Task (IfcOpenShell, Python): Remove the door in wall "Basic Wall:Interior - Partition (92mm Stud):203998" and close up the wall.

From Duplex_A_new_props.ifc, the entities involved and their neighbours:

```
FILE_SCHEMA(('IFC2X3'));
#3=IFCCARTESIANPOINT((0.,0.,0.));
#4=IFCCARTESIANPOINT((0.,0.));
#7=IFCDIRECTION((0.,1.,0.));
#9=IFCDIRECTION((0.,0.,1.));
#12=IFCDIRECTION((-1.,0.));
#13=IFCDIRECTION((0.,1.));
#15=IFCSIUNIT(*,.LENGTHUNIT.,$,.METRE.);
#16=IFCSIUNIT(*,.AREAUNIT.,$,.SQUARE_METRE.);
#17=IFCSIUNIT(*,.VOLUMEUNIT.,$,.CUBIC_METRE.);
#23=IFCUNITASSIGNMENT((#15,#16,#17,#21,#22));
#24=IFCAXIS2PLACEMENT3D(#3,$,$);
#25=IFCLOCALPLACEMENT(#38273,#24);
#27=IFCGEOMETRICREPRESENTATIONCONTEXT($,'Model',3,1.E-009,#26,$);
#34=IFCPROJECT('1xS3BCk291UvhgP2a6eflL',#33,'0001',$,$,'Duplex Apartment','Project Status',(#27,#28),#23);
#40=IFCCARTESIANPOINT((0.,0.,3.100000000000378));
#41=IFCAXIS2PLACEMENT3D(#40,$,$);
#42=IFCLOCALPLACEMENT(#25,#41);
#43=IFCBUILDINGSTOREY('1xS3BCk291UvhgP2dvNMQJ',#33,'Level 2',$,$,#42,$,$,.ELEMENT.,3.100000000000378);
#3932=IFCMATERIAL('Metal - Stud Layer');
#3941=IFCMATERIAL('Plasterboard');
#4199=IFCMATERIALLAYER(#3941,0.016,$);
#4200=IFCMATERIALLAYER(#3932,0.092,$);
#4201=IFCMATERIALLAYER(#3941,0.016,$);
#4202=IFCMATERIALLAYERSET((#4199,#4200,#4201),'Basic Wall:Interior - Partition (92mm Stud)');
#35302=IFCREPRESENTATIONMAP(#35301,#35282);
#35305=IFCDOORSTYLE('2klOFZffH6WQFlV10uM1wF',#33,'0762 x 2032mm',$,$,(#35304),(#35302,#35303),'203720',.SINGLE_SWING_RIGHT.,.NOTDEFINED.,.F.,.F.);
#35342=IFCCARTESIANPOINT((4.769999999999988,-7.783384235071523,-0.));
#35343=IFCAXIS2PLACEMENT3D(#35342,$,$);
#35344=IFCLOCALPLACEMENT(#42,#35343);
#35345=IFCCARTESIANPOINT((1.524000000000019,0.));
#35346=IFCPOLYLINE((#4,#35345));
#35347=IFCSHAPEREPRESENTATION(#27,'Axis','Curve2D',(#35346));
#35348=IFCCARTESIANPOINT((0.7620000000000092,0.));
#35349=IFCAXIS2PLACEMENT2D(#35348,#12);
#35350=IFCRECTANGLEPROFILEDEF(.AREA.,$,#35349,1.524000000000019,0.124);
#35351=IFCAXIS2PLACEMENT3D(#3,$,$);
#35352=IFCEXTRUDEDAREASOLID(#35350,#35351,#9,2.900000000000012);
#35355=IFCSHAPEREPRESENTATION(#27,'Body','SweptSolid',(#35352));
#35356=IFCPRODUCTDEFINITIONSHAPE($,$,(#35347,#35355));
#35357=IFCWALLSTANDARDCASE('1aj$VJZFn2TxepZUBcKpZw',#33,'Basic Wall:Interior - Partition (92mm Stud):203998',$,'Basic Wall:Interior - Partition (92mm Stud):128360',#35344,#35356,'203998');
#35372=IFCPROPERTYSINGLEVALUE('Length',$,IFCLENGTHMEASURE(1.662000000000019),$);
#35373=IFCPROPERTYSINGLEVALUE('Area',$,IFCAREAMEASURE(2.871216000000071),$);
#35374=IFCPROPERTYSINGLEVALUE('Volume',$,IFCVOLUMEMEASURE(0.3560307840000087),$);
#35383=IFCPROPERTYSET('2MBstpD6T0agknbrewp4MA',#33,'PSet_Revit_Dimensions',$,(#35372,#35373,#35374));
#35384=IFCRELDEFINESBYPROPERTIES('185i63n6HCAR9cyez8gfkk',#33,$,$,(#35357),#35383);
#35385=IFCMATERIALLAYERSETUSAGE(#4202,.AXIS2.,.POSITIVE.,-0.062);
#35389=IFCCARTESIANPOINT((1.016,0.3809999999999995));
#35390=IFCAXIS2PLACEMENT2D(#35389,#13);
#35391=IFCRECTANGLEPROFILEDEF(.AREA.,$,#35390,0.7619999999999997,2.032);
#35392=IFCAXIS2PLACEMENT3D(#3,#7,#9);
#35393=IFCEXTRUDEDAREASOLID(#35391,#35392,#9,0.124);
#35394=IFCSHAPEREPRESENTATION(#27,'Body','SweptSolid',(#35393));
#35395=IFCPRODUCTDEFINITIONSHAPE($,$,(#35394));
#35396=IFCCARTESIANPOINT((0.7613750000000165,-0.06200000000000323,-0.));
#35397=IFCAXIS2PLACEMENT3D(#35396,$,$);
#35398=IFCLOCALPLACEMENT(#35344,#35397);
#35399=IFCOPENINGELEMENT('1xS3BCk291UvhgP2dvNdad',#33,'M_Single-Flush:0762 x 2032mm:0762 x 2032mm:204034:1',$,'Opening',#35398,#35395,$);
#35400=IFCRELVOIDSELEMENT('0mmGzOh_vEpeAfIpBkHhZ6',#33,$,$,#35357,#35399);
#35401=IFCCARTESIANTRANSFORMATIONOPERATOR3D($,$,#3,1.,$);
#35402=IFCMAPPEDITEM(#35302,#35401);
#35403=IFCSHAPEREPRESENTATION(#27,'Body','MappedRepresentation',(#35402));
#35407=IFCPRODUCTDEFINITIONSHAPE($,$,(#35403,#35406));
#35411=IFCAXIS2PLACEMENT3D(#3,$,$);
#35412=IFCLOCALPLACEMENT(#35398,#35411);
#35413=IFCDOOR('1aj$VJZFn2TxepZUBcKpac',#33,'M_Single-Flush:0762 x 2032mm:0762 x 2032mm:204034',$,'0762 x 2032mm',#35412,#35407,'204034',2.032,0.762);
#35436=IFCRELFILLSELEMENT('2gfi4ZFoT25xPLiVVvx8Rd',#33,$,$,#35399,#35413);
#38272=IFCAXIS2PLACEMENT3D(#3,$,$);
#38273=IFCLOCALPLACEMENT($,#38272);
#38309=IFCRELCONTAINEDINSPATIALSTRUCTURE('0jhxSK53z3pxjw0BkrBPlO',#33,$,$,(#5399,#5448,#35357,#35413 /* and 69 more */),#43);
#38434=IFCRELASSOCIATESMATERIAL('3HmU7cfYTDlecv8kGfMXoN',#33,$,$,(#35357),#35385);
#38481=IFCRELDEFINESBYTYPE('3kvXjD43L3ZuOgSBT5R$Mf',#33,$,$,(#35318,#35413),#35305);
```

```python
import ifcopenshell
import ifcopenshell.api.feature
import ifcopenshell.api.pset
import ifcopenshell.api.root
import ifcopenshell.geom
import ifcopenshell.util.element
import ifcopenshell.util.shape
import ifcopenshell.util.unit

model = ifcopenshell.open("Duplex_A_new_props.ifc")
area_scale = ifcopenshell.util.unit.calculate_unit_scale(model, "AREAUNIT")
volume_scale = ifcopenshell.util.unit.calculate_unit_scale(model, "VOLUMEUNIT")
settings = ifcopenshell.geom.settings()


def volume(element):
    """Net volume in cubic metres, openings subtracted."""
    shape = ifcopenshell.geom.create_shape(settings, element)
    return ifcopenshell.util.shape.get_volume(shape.geometry)


door = model.by_guid("1aj$VJZFn2TxepZUBcKpac")
opening = door.FillsVoids[0].RelatingOpeningElement
wall = opening.VoidsElements[0].RelatingBuildingElement
before = volume(wall)

ifcopenshell.api.root.remove_product(model, product=door)
ifcopenshell.api.feature.remove_feature(model, feature=opening)

after = volume(wall)
thickness = 0.124  # wall thickness in metres

# Update the wall's stored quantities.
pset = model.by_id(ifcopenshell.util.element.get_pset(wall, "PSet_Revit_Dimensions", should_inherit=False)["id"])
ifcopenshell.api.pset.edit_pset(model, pset=pset, properties={
    "Area": model.create_entity("IfcAreaMeasure", after / thickness / area_scale),
    "Volume": model.create_entity("IfcVolumeMeasure", after / volume_scale),
})

print(f"wall volume {before:.3f} -> {after:.3f} m3")

model.write("Duplex_A_new_props_updated.ifc")
```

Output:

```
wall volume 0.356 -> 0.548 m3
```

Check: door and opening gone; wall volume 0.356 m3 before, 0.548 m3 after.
